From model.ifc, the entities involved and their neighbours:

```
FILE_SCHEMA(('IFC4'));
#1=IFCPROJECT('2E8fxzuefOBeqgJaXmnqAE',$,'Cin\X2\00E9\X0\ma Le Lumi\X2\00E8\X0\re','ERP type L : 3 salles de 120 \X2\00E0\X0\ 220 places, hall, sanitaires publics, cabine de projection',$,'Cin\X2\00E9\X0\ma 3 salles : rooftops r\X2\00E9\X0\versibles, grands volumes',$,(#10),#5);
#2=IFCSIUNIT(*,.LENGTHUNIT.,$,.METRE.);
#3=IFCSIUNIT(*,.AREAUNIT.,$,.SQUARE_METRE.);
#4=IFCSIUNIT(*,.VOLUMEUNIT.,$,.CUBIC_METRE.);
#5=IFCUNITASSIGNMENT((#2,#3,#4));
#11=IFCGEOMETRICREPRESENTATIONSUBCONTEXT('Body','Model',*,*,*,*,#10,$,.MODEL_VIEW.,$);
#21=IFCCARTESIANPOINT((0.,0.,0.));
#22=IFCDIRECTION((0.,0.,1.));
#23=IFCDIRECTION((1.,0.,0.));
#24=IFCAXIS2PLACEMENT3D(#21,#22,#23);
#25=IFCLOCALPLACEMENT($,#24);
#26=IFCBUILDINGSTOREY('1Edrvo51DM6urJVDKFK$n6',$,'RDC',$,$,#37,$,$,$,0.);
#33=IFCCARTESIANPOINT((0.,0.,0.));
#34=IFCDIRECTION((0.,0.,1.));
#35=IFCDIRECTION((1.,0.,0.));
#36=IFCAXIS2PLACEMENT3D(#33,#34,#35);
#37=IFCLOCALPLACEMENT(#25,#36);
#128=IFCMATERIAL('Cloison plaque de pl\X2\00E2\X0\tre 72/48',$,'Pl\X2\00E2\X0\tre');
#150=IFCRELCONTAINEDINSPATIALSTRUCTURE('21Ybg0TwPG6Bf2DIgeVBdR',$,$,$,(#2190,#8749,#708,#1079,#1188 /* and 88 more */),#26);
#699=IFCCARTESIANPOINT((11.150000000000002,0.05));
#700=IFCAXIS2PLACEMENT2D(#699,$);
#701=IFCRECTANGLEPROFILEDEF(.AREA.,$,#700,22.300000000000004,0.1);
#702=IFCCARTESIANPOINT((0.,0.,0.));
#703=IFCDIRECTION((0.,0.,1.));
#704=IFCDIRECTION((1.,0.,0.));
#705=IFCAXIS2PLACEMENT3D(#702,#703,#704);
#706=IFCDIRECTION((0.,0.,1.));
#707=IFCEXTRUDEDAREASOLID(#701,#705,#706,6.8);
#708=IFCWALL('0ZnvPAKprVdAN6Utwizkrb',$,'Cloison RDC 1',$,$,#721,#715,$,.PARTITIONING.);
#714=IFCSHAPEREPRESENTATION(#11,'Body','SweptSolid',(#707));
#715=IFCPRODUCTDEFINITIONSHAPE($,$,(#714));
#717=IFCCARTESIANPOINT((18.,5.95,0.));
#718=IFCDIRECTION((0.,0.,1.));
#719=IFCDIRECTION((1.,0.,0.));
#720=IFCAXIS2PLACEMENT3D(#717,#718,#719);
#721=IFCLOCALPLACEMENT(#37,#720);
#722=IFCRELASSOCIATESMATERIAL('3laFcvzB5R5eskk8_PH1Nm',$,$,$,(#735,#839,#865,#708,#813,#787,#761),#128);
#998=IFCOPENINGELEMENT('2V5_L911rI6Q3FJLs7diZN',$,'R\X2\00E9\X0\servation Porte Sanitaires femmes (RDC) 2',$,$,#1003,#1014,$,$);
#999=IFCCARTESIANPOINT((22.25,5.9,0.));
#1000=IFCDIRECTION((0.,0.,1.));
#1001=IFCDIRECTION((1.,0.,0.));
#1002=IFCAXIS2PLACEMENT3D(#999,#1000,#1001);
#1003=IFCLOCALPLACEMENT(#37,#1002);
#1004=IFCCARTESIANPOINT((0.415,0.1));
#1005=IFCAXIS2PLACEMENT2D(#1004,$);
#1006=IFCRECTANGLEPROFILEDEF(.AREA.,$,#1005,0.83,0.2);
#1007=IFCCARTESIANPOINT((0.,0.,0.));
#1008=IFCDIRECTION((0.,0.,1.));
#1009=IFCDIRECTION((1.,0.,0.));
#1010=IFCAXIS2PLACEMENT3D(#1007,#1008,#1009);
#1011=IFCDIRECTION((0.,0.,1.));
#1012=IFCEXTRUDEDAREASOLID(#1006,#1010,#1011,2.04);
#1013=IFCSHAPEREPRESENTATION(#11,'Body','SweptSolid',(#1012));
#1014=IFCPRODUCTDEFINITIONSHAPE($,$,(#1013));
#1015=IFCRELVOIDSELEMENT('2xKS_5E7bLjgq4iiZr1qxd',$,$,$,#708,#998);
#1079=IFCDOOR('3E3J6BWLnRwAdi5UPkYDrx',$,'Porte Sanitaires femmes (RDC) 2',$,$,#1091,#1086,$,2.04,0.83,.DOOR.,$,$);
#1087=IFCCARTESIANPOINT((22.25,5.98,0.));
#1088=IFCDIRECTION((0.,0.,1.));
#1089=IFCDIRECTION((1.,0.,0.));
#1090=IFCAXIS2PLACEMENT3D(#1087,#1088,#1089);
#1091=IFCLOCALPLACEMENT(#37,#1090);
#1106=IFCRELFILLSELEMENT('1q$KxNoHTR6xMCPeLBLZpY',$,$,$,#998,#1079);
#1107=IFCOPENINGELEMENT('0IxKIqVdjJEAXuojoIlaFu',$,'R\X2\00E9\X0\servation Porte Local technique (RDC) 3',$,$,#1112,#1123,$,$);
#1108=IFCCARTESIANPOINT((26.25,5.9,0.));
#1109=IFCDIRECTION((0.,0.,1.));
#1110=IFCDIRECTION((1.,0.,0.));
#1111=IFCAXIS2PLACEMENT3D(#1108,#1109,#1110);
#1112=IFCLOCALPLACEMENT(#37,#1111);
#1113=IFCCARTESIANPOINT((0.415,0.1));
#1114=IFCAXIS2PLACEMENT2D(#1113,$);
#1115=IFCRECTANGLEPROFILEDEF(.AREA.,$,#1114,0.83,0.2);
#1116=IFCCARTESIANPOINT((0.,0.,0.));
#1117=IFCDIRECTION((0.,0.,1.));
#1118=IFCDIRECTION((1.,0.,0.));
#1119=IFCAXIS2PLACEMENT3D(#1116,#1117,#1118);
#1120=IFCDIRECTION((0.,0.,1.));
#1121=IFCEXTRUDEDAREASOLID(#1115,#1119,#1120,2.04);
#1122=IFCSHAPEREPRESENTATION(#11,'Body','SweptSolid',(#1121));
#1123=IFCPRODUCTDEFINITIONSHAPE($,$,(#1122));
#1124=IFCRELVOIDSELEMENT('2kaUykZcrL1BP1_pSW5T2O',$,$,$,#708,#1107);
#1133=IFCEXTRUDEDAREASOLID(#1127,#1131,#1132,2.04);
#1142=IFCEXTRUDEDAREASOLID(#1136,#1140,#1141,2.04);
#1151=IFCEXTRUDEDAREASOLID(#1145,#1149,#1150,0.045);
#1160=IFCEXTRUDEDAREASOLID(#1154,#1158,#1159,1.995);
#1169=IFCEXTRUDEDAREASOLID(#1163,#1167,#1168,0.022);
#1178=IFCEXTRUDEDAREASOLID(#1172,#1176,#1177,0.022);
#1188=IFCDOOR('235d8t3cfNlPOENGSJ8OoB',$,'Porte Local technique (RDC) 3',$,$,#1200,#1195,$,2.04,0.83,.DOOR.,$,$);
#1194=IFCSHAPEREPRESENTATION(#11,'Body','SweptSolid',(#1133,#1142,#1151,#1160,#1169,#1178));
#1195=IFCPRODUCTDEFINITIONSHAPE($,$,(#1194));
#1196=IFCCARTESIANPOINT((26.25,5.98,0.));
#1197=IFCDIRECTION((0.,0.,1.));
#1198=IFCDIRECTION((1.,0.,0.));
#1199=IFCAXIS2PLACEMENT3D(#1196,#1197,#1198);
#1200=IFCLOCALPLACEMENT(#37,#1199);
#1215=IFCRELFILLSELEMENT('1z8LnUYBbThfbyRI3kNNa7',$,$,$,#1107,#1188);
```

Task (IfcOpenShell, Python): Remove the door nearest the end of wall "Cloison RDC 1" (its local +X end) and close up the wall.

```python
import ifcopenshell
import ifcopenshell.api.feature
import ifcopenshell.api.root
import ifcopenshell.geom
import ifcopenshell.util.shape

model = ifcopenshell.open("model.ifc")
settings = ifcopenshell.geom.settings()


def volume(element):
    """Net volume in cubic metres, openings subtracted."""
    shape = ifcopenshell.geom.create_shape(settings, element)
    return ifcopenshell.util.shape.get_volume(shape.geometry)


door = model.by_guid("235d8t3cfNlPOENGSJ8OoB")
opening = door.FillsVoids[0].RelatingOpeningElement
wall = opening.VoidsElements[0].RelatingBuildingElement
before = volume(wall)

ifcopenshell.api.root.remove_product(model, product=door)
ifcopenshell.api.feature.remove_feature(model, feature=opening)

after = volume(wall)

print(f"wall volume {before:.3f} -> {after:.3f} m3")

model.write("model_updated.ifc")
```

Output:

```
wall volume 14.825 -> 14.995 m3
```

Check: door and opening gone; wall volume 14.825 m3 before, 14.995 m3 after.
